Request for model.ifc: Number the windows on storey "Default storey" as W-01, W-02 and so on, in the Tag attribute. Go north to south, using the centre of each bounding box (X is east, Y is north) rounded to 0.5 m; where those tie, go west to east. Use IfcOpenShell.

First a look at what the model holds.

```python
import ifcopenshell
import ifcopenshell.util.element
import ifcopenshell.util.placement

model = ifcopenshell.open("model.ifc")
print(model.schema)
storey = next(s for s in model.by_type("IfcBuildingStorey") if s.Name == "Default storey")
windows = [e for e in ifcopenshell.util.element.get_decomposition(storey) if e.is_a("IfcWindow")]
for e in sorted(windows, key=lambda e: e.id()):
    origin = ifcopenshell.util.placement.get_local_placement(e.ObjectPlacement)[:3, 3]
    print(e.id(), e.Tag, e.Name, origin.round(2) + 0.0, sep=" | ")
```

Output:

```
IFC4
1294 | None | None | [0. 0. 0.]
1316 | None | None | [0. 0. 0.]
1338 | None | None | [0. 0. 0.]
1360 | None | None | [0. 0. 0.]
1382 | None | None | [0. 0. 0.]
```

```python
import ifcopenshell
import ifcopenshell.geom
import ifcopenshell.util.element
import ifcopenshell.util.shape

model = ifcopenshell.open("model.ifc")
settings = ifcopenshell.geom.settings()
settings.set("use-world-coords", True)


def centre(element):
    shape = ifcopenshell.geom.create_shape(settings, element)
    return ifcopenshell.util.shape.get_bbox_centroid(shape.geometry)


storey = next(s for s in model.by_type("IfcBuildingStorey") if s.Name == "Default storey")
windows = [e for e in ifcopenshell.util.element.get_decomposition(storey) if e.is_a("IfcWindow")]

# Insertion points can sit at a corner or the storey origin, so sort by the geometry (in metres).
centres = {e: centre(e) for e in windows}
windows.sort(key=lambda e: (-round(centres[e][1] / 0.5), centres[e][0]))

for i, e in enumerate(windows, start=1):
    number = f"W-{i:02d}"
    e.Tag = number
    print(e.id(), number)

model.write("model-out.ifc")
```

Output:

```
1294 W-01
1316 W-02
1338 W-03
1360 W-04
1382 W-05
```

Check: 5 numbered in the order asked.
